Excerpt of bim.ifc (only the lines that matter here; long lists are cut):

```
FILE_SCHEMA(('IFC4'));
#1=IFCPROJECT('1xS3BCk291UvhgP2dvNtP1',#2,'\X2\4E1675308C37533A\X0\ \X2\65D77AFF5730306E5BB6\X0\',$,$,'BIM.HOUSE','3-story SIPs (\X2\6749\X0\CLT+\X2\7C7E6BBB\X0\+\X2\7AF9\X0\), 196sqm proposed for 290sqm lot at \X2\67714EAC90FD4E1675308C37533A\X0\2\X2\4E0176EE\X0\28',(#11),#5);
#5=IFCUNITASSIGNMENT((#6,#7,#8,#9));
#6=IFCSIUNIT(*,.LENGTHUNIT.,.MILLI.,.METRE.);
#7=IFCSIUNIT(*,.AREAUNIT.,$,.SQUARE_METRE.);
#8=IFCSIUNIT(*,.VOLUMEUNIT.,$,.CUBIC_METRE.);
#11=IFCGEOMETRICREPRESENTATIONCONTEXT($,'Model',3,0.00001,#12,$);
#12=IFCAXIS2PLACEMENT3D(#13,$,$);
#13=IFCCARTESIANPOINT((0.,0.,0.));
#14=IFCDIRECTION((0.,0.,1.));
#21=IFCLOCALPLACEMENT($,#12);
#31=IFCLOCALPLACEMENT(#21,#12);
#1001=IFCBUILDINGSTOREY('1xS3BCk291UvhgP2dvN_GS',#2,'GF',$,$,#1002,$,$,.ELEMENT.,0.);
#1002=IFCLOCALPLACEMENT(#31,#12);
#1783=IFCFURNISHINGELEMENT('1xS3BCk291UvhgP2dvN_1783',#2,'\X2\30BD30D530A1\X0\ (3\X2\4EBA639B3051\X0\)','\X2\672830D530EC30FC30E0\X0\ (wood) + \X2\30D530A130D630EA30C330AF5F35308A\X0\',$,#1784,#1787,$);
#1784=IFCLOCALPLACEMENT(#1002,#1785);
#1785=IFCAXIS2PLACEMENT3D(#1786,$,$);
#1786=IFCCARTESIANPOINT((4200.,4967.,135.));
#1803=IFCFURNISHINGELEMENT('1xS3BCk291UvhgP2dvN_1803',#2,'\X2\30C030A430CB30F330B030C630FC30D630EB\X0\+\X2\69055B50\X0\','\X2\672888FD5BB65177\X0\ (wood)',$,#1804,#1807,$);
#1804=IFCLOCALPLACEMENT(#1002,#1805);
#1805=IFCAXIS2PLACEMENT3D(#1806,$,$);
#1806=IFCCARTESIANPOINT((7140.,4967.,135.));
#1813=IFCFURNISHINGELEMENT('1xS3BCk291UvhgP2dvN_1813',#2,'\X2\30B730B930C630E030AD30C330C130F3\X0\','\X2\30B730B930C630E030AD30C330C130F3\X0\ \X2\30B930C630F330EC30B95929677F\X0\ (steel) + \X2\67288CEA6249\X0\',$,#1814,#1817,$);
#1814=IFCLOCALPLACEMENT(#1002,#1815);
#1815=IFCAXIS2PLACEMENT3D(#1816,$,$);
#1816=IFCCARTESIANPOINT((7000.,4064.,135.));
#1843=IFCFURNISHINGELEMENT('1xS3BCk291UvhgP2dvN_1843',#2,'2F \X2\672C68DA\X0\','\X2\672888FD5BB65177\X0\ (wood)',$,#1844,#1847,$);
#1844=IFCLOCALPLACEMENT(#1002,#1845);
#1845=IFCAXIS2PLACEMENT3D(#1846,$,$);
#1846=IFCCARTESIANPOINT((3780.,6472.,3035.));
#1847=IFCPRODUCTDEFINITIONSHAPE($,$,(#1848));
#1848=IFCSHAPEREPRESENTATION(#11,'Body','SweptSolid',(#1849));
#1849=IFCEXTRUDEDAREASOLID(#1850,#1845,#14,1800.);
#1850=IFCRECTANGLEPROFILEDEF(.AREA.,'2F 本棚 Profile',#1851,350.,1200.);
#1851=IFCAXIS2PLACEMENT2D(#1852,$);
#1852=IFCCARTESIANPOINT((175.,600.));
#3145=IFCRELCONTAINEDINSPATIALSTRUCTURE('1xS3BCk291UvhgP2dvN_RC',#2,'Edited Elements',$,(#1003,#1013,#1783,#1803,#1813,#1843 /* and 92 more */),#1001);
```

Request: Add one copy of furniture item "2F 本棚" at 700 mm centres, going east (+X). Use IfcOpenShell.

```python
import numpy as np
import ifcopenshell
import ifcopenshell.api.geometry
import ifcopenshell.api.root
import ifcopenshell.util.element
import ifcopenshell.util.placement

model = ifcopenshell.open("bim.ifc")


def reuse_history(source, copy):
    """copy_class also copies each property set's owner history, people and application; keep the originals."""
    for rel in copy.IsDefinedBy:
        if rel.is_a("IfcRelDefinesByProperties") and (history := rel.RelatingPropertyDefinition.OwnerHistory):
            rel.RelatingPropertyDefinition.OwnerHistory = source.OwnerHistory
            ifcopenshell.util.element.remove_deep2(model, history)


source = model.by_guid("1xS3BCk291UvhgP2dvN_1843")
base = ifcopenshell.util.placement.get_local_placement(source.ObjectPlacement)
step = np.array([1.0, 0.0, 0.0]) * 700.0

for i in range(1, 2):
    copy = ifcopenshell.api.root.copy_class(model, product=source)
    copy.Representation = ifcopenshell.util.element.copy_deep(
        model, source.Representation, exclude=["IfcGeometricRepresentationContext", "IfcRepresentationMap"]
    )
    reuse_history(source, copy)
    matrix = base.copy()
    matrix[:3, 3] += i * step
    print("added at", matrix[:3, 3].round(3) + 0.0)
    ifcopenshell.api.geometry.edit_object_placement(model, product=copy, matrix=matrix, is_si=False)

model.write("bim-out.ifc")
```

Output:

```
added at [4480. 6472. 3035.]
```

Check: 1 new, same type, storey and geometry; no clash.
